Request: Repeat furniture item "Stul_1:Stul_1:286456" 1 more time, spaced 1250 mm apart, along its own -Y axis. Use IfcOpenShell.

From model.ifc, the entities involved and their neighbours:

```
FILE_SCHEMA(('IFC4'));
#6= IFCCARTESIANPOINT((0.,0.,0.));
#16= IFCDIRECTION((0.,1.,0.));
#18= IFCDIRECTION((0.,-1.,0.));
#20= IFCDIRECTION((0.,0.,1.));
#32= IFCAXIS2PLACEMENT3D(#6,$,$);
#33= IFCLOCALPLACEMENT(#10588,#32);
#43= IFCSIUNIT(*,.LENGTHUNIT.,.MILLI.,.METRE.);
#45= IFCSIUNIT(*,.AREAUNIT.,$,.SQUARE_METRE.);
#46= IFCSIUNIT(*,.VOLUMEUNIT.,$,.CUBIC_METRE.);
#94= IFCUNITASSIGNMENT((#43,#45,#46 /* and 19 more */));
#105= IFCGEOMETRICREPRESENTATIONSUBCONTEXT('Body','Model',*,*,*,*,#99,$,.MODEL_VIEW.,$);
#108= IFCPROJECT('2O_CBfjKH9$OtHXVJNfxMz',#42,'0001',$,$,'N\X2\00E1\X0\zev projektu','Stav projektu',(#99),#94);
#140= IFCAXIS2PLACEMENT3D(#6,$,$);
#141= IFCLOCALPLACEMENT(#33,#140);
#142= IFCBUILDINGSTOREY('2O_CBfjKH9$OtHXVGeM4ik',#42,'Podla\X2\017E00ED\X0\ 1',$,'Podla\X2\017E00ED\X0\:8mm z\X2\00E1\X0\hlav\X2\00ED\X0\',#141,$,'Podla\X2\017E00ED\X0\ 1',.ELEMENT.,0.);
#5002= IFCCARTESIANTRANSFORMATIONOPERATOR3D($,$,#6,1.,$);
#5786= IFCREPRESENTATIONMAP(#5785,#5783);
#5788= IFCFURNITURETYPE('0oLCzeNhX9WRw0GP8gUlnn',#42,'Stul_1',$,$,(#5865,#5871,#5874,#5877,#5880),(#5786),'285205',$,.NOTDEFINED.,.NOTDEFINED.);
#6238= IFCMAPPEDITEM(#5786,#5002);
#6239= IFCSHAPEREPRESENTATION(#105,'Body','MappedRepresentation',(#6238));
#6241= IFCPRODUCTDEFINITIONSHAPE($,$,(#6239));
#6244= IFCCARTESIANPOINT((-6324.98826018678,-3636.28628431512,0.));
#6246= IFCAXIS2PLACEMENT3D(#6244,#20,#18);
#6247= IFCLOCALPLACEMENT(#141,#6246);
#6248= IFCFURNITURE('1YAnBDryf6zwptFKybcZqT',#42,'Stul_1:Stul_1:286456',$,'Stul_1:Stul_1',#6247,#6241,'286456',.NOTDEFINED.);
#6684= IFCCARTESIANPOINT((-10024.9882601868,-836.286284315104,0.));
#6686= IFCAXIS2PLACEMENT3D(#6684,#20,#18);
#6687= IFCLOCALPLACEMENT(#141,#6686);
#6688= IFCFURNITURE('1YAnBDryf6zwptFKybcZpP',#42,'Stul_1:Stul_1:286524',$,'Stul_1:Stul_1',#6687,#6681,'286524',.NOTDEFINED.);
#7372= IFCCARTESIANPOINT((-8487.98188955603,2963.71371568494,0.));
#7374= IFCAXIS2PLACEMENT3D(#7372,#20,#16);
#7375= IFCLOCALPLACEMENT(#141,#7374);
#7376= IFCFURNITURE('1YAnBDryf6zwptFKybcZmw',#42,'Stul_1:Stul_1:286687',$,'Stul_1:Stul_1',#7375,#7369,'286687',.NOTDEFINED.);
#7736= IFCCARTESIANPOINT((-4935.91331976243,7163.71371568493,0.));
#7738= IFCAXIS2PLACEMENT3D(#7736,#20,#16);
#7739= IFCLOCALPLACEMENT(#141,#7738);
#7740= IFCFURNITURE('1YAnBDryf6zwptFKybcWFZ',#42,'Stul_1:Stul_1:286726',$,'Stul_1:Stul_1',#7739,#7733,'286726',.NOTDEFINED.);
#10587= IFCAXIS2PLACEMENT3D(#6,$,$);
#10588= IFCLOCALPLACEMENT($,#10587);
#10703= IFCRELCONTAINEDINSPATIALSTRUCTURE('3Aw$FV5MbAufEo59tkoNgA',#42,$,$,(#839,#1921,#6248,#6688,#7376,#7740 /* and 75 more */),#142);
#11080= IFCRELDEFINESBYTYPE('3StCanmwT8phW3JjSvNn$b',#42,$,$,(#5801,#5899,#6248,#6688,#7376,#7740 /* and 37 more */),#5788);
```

```python
import ifcopenshell
import ifcopenshell.api.geometry
import ifcopenshell.api.root
import ifcopenshell.util.element
import ifcopenshell.util.placement
import ifcopenshell.util.unit

model = ifcopenshell.open("model.ifc")
unit_scale = ifcopenshell.util.unit.calculate_unit_scale(model)


def reuse_history(source, copy):
    """copy_class also copies each property set's owner history, people and application; keep the originals."""
    for rel in copy.IsDefinedBy:
        if rel.is_a("IfcRelDefinesByProperties") and (history := rel.RelatingPropertyDefinition.OwnerHistory):
            rel.RelatingPropertyDefinition.OwnerHistory = source.OwnerHistory
            ifcopenshell.util.element.remove_deep2(model, history)


source = model.by_guid("1YAnBDryf6zwptFKybcZqT")
base = ifcopenshell.util.placement.get_local_placement(source.ObjectPlacement)
step = -base[:3, 1] * 1.25 / unit_scale

for i in range(1, 2):
    copy = ifcopenshell.api.root.copy_class(model, product=source)
    copy.Representation = ifcopenshell.util.element.copy_deep(
        model, source.Representation, exclude=["IfcGeometricRepresentationContext", "IfcRepresentationMap"]
    )
    copy.Name = "Stul_1:Stul_1"
    copy.Tag = None
    reuse_history(source, copy)
    matrix = base.copy()
    matrix[:3, 3] += i * step
    print("added at", matrix[:3, 3].round(3) + 0.0)
    ifcopenshell.api.geometry.edit_object_placement(model, product=copy, matrix=matrix, is_si=False)

model.write("model_edited.ifc")
```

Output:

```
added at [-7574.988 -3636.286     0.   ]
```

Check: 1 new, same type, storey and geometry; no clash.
